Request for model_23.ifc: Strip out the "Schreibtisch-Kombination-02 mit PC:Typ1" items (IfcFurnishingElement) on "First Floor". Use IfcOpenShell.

First a look at what the model holds.

```python
import ifcopenshell
import ifcopenshell.util.element

model = ifcopenshell.open("model_23.ifc")
print(model.schema)
storey = next(s for s in model.by_type("IfcBuildingStorey") if s.Name == "First Floor")
furniture = [e for e in ifcopenshell.util.element.get_decomposition(storey) if e.is_a("IfcFurnishingElement")]
seen = {}
for e in furniture:
    element_type = ifcopenshell.util.element.get_type(e)
    name = element_type.Name if element_type not in (None, e) else None
    seen[name] = seen.get(name, 0) + 1
for name, count in sorted(seen.items(), key=str):
    print(count, "x", name)
```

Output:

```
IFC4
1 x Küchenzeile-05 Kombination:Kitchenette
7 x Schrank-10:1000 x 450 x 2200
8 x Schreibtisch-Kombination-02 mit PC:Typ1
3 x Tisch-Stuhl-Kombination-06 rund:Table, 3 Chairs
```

```python
import ifcopenshell
import ifcopenshell.api.root
import ifcopenshell.util.element

model = ifcopenshell.open("model_23.ifc")

storey = next(s for s in model.by_type("IfcBuildingStorey") if s.Name == "First Floor")
furniture = [e for e in ifcopenshell.util.element.get_decomposition(storey) if e.is_a("IfcFurnishingElement")]
targets = [e for e in furniture if (t := ifcopenshell.util.element.get_type(e)) not in (None, e) and t.Name == "Schreibtisch-Kombination-02 mit PC:Typ1"]

for e in targets:
    ifcopenshell.api.root.remove_product(model, product=e)
print(len(targets), "removed")

model.write("model_23_v2.ifc")
```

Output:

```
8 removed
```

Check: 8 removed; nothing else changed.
